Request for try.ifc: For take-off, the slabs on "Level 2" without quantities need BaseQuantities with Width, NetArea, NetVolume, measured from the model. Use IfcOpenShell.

First a look at what the model holds.

```python
import ifcopenshell
import ifcopenshell.util.element
import ifcopenshell.util.unit

model = ifcopenshell.open("try.ifc")
print(model.schema)
for unit_type in ("LENGTHUNIT", "AREAUNIT", "VOLUMEUNIT"):
    print(unit_type, ifcopenshell.util.unit.calculate_unit_scale(model, unit_type))
storey = next(s for s in model.by_type("IfcBuildingStorey") if s.Name == "Level 2")
slabs = [e for e in ifcopenshell.util.element.get_decomposition(storey) if e.is_a("IfcSlab")]
for e in sorted(slabs, key=lambda e: e.id()):
    print(e.id(), e.is_a(), e.Name, list(ifcopenshell.util.element.get_psets(e, qtos_only=True)), sep=" | ")
```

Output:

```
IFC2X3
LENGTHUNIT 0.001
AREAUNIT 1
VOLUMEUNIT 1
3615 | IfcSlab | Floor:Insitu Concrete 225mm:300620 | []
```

```python
import ifcopenshell
import ifcopenshell.api.pset
import ifcopenshell.geom
import ifcopenshell.util.element
import ifcopenshell.util.shape
import ifcopenshell.util.unit

model = ifcopenshell.open("try.ifc")
unit_scale = ifcopenshell.util.unit.calculate_unit_scale(model)
area_scale = ifcopenshell.util.unit.calculate_unit_scale(model, "AREAUNIT")
volume_scale = ifcopenshell.util.unit.calculate_unit_scale(model, "VOLUMEUNIT")
settings = ifcopenshell.geom.settings()

storey = next(s for s in model.by_type("IfcBuildingStorey") if s.Name == "Level 2")
slabs = [e for e in ifcopenshell.util.element.get_decomposition(storey) if e.is_a("IfcSlab")]

for e in sorted(slabs, key=lambda e: e.id()):
    if ifcopenshell.util.element.get_psets(e, qtos_only=True, should_inherit=False):
        continue
    # Geometry comes back in metres, in the element's own axes.
    shape = ifcopenshell.geom.create_shape(settings, e)
    values = {
        "Width": ifcopenshell.util.shape.get_z(shape.geometry) / unit_scale,
        "NetArea": ifcopenshell.util.shape.get_footprint_area(shape.geometry) / area_scale,
        "NetVolume": ifcopenshell.util.shape.get_volume(shape.geometry) / volume_scale,
    }
    qto = ifcopenshell.api.pset.add_qto(model, product=e, name="BaseQuantities")
    ifcopenshell.api.pset.edit_qto(model, qto=qto, properties=values)
    print(e.id(), {k: round(v, 3) for k, v in values.items()})

model.write("try_updated.ifc")
```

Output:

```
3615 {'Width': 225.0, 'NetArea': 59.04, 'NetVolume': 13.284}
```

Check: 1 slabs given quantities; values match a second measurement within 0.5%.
